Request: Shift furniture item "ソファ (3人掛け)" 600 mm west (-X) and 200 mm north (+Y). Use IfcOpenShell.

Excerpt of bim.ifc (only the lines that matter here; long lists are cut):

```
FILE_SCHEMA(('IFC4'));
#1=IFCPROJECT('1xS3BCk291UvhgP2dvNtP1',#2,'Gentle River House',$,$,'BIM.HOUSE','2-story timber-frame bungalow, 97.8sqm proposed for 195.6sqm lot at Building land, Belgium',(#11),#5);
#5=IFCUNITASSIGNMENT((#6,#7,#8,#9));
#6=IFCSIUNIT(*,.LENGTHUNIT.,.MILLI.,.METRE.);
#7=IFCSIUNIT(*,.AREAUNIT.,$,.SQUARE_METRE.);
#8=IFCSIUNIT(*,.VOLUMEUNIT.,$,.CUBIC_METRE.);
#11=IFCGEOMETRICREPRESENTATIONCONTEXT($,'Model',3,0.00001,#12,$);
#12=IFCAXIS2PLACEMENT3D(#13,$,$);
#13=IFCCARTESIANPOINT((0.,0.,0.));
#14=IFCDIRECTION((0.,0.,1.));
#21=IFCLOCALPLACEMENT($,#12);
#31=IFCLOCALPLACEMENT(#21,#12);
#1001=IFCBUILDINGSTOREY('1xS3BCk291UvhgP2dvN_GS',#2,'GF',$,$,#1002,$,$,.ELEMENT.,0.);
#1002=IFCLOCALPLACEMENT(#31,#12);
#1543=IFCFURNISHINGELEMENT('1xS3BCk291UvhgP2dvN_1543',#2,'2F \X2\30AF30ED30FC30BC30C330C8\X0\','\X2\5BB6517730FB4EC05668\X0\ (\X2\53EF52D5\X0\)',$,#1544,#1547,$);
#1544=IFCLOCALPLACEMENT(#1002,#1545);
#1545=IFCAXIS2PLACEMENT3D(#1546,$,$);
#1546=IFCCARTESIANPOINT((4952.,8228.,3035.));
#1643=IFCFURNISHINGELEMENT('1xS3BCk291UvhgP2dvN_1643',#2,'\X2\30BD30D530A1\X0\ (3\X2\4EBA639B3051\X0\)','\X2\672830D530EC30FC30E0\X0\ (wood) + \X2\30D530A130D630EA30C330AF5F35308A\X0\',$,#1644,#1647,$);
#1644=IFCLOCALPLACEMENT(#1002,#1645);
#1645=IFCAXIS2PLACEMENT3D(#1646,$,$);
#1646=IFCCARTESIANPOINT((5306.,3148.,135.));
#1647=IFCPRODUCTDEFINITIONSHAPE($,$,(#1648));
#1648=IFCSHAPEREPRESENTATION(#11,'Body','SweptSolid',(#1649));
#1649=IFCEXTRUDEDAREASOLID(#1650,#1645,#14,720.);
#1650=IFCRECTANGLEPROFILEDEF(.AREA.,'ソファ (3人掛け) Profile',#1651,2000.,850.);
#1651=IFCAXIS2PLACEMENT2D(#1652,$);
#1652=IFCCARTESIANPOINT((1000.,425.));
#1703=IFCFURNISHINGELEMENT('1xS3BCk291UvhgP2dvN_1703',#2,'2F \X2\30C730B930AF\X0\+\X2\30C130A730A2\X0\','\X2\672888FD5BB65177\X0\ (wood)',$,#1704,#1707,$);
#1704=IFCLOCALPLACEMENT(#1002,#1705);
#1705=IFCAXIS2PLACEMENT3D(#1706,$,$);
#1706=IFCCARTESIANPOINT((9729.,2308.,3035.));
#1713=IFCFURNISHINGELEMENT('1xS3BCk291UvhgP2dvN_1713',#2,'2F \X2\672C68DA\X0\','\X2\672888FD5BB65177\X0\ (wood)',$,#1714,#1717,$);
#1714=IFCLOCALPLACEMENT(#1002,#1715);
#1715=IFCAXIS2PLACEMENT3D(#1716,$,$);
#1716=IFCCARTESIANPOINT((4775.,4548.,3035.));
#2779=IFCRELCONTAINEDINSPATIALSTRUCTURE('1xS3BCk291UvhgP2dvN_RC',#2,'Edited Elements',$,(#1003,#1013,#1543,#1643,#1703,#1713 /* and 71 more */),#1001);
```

```python
import ifcopenshell
import ifcopenshell.api.geometry
import ifcopenshell.util.placement

model = ifcopenshell.open("bim.ifc")

item = model.by_guid("1xS3BCk291UvhgP2dvN_1643")
matrix = ifcopenshell.util.placement.get_local_placement(item.ObjectPlacement)
matrix[0, 3] -= 600.0
matrix[1, 3] += 200.0
ifcopenshell.api.geometry.edit_object_placement(model, product=item, matrix=matrix, is_si=False)

print(ifcopenshell.util.placement.get_local_placement(item.ObjectPlacement).round(3) + 0.0)

model.write("bim-out.ifc")
```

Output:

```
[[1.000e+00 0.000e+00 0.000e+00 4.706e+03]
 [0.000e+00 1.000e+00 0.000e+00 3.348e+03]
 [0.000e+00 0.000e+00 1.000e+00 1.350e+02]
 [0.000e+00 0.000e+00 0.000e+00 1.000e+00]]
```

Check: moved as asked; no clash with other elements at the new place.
